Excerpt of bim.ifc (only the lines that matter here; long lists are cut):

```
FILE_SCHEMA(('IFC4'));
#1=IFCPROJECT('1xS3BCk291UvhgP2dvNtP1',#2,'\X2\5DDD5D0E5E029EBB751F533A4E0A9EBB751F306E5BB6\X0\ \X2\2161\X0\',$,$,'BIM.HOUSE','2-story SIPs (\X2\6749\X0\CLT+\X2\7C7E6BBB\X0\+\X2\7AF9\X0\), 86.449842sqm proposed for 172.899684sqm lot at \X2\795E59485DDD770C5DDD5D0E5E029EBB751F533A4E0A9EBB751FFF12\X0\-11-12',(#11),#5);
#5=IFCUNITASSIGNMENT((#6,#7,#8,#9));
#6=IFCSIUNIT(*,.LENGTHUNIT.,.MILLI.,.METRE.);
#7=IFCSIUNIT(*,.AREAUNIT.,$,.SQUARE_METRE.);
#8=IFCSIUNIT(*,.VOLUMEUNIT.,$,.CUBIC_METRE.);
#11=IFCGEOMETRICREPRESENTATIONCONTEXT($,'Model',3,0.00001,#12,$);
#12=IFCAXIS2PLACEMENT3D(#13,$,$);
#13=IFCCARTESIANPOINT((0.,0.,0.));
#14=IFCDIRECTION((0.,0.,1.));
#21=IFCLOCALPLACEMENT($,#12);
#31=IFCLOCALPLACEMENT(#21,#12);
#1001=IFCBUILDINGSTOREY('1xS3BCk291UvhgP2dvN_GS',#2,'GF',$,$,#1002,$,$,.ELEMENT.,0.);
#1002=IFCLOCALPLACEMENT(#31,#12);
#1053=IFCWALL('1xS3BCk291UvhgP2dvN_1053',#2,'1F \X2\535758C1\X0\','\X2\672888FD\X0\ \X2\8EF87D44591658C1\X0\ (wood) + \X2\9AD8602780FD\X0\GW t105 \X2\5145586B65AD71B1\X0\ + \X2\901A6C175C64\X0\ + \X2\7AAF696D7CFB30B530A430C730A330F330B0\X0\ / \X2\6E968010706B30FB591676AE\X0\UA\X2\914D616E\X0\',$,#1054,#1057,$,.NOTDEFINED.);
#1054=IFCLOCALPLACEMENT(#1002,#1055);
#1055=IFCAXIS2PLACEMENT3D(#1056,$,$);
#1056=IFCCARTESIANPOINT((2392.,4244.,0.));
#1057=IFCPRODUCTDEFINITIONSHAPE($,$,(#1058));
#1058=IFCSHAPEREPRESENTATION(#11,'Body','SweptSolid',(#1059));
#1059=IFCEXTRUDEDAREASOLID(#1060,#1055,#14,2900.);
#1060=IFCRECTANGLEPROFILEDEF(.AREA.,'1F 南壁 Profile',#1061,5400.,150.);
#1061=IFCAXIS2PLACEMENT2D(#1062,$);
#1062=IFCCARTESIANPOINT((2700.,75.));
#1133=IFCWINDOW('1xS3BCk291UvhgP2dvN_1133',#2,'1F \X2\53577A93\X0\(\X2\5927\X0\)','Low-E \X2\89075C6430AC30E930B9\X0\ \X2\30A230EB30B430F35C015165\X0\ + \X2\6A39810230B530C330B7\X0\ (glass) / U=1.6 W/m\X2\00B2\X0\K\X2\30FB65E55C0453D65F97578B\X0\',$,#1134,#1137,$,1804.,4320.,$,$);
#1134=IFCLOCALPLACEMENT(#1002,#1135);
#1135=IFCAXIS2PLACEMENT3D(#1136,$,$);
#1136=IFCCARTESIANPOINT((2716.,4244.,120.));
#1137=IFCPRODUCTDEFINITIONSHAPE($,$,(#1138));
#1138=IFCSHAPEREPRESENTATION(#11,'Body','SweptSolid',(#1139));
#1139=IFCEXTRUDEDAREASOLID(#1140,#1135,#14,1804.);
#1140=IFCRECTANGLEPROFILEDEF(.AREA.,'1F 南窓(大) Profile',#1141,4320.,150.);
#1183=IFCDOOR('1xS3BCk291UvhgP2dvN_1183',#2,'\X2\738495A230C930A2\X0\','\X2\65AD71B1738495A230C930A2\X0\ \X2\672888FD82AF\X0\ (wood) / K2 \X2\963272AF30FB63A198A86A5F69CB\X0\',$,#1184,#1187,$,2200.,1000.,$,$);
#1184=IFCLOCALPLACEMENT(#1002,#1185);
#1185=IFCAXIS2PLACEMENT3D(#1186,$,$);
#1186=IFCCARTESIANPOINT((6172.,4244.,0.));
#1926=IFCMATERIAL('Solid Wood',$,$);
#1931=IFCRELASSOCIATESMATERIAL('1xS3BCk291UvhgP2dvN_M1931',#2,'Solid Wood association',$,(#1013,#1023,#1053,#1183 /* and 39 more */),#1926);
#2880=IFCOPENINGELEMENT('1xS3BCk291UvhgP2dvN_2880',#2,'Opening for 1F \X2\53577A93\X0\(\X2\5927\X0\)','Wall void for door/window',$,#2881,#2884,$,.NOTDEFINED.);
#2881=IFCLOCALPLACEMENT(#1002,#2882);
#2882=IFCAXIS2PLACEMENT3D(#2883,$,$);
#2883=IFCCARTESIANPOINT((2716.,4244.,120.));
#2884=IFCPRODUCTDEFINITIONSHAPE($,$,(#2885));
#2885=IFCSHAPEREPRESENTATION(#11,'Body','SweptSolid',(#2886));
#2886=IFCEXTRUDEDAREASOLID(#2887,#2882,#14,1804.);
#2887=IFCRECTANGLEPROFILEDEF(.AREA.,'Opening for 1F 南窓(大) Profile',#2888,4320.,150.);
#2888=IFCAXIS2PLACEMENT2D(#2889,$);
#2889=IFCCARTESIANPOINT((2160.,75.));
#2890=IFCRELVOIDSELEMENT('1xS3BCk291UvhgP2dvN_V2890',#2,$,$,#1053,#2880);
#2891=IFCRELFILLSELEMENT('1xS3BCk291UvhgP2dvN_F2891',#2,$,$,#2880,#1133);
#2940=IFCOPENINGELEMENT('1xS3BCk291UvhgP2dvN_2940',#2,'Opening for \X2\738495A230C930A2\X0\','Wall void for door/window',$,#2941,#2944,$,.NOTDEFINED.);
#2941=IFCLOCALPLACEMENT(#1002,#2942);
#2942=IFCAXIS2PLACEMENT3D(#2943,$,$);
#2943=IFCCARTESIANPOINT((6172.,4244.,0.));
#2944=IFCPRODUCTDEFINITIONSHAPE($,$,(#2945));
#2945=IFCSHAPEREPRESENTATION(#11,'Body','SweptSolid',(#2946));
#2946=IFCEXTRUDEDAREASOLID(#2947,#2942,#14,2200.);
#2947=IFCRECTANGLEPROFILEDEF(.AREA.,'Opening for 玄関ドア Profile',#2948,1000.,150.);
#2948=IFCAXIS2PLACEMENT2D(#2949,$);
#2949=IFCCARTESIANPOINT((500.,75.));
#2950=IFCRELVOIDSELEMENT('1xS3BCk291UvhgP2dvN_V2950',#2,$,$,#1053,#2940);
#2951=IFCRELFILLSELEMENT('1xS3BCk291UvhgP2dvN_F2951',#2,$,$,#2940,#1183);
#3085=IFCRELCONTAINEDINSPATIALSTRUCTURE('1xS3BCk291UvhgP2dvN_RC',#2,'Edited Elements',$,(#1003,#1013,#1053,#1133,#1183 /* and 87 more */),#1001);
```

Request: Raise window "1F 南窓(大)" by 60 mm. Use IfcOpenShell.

```python
import numpy as np
import ifcopenshell
import ifcopenshell.api.geometry
import ifcopenshell.util.placement
import ifcopenshell.util.unit

model = ifcopenshell.open("bim.ifc")
unit_scale = ifcopenshell.util.unit.calculate_unit_scale(model)

window = model.by_guid("1xS3BCk291UvhgP2dvN_1133")
opening = window.FillsVoids[0].RelatingOpeningElement
dz = 0.06 / unit_scale

shift = np.array([0.0, 0.0, dz])
# The window is not placed relative to its opening, so move both.
for product in (opening, window):
    matrix = ifcopenshell.util.placement.get_local_placement(product.ObjectPlacement)
    matrix[:3, 3] += shift
    ifcopenshell.api.geometry.edit_object_placement(model, product=product, matrix=matrix, is_si=False)

print(f"moved by {dz * unit_scale:+.3f} m")

model.write("bim-out.ifc")
```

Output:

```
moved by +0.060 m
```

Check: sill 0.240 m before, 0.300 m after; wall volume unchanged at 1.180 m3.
